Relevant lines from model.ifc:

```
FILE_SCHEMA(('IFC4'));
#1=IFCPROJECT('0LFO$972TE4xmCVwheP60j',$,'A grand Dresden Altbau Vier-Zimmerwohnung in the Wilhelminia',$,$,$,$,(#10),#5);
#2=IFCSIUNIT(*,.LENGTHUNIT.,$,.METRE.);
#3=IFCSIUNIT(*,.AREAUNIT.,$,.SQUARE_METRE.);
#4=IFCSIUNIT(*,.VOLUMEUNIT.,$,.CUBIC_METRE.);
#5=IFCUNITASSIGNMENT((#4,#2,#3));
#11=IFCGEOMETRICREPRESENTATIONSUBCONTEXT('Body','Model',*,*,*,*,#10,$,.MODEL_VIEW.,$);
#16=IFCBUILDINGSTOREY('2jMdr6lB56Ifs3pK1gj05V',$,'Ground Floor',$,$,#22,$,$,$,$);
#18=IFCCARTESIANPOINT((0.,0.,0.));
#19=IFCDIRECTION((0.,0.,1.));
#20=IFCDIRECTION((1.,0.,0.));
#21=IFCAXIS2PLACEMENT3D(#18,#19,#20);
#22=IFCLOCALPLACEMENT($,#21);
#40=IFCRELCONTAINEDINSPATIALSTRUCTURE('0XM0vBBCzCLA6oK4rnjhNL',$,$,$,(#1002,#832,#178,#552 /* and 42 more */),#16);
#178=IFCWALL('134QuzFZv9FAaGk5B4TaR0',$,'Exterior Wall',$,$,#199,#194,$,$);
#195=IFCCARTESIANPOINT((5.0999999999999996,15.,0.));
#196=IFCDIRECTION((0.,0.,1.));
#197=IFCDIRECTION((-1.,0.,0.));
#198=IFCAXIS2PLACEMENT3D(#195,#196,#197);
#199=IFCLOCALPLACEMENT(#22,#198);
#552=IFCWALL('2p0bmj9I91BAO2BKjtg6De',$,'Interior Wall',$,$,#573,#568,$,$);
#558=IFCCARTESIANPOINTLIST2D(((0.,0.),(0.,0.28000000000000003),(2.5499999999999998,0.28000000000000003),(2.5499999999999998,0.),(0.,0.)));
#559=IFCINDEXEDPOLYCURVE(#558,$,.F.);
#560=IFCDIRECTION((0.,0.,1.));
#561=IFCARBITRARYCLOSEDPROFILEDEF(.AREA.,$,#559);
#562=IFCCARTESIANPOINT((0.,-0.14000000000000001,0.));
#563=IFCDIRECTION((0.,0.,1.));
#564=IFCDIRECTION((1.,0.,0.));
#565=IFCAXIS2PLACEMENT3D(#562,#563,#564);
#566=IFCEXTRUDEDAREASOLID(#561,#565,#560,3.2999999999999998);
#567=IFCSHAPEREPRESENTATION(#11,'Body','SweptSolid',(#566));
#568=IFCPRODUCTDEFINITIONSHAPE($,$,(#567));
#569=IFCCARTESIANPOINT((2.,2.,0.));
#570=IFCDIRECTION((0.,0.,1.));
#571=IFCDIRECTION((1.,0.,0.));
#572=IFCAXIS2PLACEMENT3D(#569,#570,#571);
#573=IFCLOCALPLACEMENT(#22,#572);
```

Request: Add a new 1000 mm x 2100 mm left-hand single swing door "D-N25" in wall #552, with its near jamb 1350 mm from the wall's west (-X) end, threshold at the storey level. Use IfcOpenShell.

```python
import numpy as np
import ifcopenshell
import ifcopenshell.api.feature
import ifcopenshell.api.geometry
import ifcopenshell.api.root
import ifcopenshell.api.spatial
import ifcopenshell.geom
import ifcopenshell.util.element
import ifcopenshell.util.placement
import ifcopenshell.util.representation
import ifcopenshell.util.shape
import ifcopenshell.util.unit

model = ifcopenshell.open("model.ifc")
unit_scale = ifcopenshell.util.unit.calculate_unit_scale(model)
settings = ifcopenshell.geom.settings()


def volume(element):
    """Net volume in cubic metres, openings subtracted."""
    shape = ifcopenshell.geom.create_shape(settings, element)
    return ifcopenshell.util.shape.get_volume(shape.geometry)


wall = model.by_id(552)
storey = ifcopenshell.util.element.get_container(wall, ifc_class="IfcBuildingStorey")
context = ifcopenshell.util.representation.get_context(model, "Model", "Body", "MODEL_VIEW")
before = volume(wall)

width, height, from_end, sill = 1, 2.1, 1.35, 0.0  # metres

# The wall runs along its own X axis, and the end named is its -X end.
wall_shape = ifcopenshell.geom.create_shape(settings, wall)
x, y, z = ifcopenshell.util.shape.get_vertices(wall_shape.geometry).T
start = x.min() + from_end
face, thickness = float(y.min()), float(y.max() - y.min())
wall_matrix = ifcopenshell.util.placement.get_local_placement(wall.ObjectPlacement)
level = ifcopenshell.util.placement.get_local_placement(storey.ObjectPlacement)[2, 3]


def in_wall(x, y):
    """Placement at x, y metres in the wall's axes, at sill height."""
    matrix = wall_matrix.copy()
    matrix[:, 3] = wall_matrix @ np.array([x / unit_scale, y / unit_scale, 0.0, 1.0])
    matrix[2, 3] = level + sill / unit_scale
    return matrix


# Opening: a box that overshoots both wall faces by 50 mm.
opening = ifcopenshell.api.root.create_entity(model, ifc_class="IfcOpeningElement", predefined_type="OPENING")
box = ifcopenshell.api.geometry.add_wall_representation(
    model, context=context, length=width, height=height, thickness=thickness + 0.1
)
ifcopenshell.api.geometry.assign_representation(model, product=opening, representation=box)
ifcopenshell.api.geometry.edit_object_placement(model, product=opening, matrix=in_wall(start, face - 0.05), is_si=False)
ifcopenshell.api.feature.add_feature(model, feature=opening, element=wall)

door = ifcopenshell.api.root.create_entity(model, ifc_class="IfcDoor", name="D-N25", predefined_type="DOOR")
door.OverallWidth, door.OverallHeight = width / unit_scale, height / unit_scale
door.OperationType = "SINGLE_SWING_LEFT"
body = ifcopenshell.api.geometry.add_door_representation(
    model,
    context=context,
    overall_width=door.OverallWidth,
    overall_height=door.OverallHeight,
    operation_type="SINGLE_SWING_LEFT",
    lining_properties={"LiningDepth": thickness / unit_scale, "ThresholdDepth": thickness / unit_scale},
)
ifcopenshell.api.geometry.assign_representation(model, product=door, representation=body)
ifcopenshell.api.spatial.assign_container(model, products=[door], relating_structure=storey)
ifcopenshell.api.feature.add_filling(model, opening=opening, element=door)

# The lining spans the wall, so the door starts at the wall face.
ifcopenshell.api.geometry.edit_object_placement(model, product=door, matrix=in_wall(start, face), is_si=False)

after = volume(wall)

print(f"wall volume {before:.3f} -> {after:.3f} m3")

model.write("model-out.ifc")
```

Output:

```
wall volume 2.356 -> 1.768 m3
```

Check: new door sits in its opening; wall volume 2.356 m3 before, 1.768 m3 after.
